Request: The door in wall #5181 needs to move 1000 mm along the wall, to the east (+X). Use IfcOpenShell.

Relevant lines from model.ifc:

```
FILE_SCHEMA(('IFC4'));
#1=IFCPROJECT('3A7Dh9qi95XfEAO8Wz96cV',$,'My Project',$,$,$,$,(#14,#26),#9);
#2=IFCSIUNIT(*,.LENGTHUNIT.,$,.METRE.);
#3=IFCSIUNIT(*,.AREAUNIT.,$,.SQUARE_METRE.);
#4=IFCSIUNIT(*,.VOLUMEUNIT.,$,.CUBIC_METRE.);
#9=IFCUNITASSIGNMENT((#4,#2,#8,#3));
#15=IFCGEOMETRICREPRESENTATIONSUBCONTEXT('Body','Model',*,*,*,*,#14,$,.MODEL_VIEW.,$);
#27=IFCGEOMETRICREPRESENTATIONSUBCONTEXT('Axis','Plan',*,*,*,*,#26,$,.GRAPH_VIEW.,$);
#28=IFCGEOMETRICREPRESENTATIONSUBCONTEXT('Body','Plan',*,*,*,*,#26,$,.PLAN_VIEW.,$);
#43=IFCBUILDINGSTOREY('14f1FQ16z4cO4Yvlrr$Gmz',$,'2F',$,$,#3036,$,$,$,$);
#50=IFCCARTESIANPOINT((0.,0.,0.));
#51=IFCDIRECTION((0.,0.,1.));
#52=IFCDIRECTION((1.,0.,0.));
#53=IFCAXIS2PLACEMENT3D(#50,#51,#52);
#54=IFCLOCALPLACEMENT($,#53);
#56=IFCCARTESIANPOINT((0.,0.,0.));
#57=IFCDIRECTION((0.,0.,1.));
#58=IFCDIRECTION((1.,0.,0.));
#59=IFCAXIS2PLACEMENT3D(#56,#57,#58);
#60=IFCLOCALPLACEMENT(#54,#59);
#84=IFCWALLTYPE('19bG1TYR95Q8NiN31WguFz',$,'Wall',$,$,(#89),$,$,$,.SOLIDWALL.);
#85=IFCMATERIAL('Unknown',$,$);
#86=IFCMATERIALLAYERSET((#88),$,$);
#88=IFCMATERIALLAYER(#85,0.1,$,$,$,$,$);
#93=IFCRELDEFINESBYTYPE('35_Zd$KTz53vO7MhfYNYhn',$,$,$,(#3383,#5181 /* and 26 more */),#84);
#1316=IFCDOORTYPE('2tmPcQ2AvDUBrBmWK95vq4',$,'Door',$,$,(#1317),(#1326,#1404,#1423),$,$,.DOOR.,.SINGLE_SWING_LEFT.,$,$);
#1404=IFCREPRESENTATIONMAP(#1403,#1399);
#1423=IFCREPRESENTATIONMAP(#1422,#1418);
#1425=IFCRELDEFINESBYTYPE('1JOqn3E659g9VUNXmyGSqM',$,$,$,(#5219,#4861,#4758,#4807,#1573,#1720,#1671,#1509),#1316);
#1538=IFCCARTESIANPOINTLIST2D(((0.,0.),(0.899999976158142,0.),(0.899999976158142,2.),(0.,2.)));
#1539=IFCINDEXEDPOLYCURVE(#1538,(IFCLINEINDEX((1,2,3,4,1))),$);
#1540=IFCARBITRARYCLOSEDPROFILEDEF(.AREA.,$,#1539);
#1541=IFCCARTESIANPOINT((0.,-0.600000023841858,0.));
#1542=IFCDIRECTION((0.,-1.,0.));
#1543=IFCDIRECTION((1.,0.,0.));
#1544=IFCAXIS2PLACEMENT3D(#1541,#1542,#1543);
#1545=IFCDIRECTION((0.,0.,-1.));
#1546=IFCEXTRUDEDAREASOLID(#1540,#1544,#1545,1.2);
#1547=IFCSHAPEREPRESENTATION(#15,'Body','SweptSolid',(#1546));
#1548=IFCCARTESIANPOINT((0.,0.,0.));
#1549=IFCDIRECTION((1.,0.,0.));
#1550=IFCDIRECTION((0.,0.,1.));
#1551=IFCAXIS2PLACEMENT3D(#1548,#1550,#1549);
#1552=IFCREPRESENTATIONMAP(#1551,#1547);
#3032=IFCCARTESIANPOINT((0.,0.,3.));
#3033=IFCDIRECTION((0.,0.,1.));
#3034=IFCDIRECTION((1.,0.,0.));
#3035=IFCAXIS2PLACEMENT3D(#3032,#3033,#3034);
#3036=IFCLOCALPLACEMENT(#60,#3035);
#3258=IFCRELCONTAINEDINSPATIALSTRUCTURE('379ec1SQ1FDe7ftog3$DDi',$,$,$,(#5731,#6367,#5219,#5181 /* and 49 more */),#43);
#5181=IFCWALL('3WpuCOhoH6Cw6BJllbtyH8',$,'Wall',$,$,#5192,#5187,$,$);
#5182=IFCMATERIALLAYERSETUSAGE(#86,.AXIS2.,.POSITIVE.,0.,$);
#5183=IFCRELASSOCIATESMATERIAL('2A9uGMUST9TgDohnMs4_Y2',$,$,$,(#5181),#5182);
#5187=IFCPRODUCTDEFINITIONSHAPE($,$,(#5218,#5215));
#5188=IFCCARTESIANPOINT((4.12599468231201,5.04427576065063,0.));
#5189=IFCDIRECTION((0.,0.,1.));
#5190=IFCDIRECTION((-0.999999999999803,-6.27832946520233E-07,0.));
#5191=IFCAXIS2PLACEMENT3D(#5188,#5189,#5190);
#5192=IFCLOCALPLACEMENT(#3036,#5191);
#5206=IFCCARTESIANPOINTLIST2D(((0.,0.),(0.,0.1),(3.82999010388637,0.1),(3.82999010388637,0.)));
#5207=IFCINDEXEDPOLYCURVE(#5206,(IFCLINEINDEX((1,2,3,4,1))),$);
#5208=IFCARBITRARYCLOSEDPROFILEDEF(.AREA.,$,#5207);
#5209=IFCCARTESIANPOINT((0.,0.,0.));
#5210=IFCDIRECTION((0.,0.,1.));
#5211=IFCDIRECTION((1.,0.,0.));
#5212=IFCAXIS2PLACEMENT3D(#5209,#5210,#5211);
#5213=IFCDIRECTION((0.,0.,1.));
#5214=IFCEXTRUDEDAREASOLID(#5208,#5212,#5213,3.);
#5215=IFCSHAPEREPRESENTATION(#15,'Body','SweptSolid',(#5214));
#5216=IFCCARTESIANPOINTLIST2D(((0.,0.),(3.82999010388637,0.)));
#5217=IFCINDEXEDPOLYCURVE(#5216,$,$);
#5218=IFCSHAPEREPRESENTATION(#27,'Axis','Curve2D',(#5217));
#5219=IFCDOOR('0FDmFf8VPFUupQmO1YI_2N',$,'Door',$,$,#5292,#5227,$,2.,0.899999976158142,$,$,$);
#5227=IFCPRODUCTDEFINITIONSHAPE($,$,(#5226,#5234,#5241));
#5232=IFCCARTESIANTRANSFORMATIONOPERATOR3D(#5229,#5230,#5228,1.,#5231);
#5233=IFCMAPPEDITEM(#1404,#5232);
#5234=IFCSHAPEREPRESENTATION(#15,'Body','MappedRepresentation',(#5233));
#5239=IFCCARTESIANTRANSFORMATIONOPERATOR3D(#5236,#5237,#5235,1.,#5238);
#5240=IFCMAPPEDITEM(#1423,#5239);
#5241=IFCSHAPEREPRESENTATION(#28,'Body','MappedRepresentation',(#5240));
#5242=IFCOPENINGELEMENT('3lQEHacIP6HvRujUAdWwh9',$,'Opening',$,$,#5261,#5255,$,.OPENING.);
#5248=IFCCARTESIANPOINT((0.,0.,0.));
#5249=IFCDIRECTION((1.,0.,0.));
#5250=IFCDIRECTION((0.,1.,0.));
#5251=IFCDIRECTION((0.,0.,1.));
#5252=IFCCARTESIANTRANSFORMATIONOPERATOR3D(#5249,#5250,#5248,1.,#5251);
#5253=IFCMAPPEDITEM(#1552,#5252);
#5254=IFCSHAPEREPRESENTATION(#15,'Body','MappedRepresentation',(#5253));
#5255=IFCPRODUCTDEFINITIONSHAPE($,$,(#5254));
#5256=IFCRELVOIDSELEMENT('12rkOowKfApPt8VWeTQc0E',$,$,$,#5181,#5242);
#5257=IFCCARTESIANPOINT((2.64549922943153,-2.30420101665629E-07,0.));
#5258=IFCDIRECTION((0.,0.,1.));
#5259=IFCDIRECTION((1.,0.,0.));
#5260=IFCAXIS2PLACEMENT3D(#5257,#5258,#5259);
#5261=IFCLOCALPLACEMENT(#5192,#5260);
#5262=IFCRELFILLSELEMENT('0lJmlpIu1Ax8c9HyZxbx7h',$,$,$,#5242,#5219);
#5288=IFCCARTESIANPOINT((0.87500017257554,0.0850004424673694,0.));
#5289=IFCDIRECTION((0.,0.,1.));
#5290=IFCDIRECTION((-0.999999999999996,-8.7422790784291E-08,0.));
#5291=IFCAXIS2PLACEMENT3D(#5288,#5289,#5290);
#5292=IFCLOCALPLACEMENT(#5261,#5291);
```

```python
import ifcopenshell
import ifcopenshell.api.geometry
import ifcopenshell.util.placement
import ifcopenshell.util.unit

model = ifcopenshell.open("model.ifc")
unit_scale = ifcopenshell.util.unit.calculate_unit_scale(model)

door = model.by_guid("0FDmFf8VPFUupQmO1YI_2N")
opening = door.FillsVoids[0].RelatingOpeningElement
wall = opening.VoidsElements[0].RelatingBuildingElement

wall_matrix = ifcopenshell.util.placement.get_local_placement(wall.ObjectPlacement)
shift = wall_matrix[:3, 0] * -1 / unit_scale
before = ifcopenshell.util.placement.get_local_placement(door.ObjectPlacement)[:3, 3].copy()

# The door is placed relative to its opening, so it follows when the opening moves.
matrix = ifcopenshell.util.placement.get_local_placement(opening.ObjectPlacement)
matrix[:3, 3] += shift
ifcopenshell.api.geometry.edit_object_placement(
    model, product=opening, matrix=matrix, is_si=False, should_transform_children=True
)

after = ifcopenshell.util.placement.get_local_placement(door.ObjectPlacement)[:3, 3]
print("door moved by", (after - before).round(3) + 0.0)

model.write("model_updated.ifc")
```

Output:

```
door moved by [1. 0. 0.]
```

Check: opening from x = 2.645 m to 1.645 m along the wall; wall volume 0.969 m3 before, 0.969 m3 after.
